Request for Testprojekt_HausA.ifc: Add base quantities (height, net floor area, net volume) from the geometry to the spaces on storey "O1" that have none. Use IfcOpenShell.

First a look at what the model holds.

```python
import ifcopenshell
import ifcopenshell.util.element
import ifcopenshell.util.unit

model = ifcopenshell.open("Testprojekt_HausA.ifc")
print(model.schema)
for unit_type in ("LENGTHUNIT", "AREAUNIT", "VOLUMEUNIT"):
    print(unit_type, ifcopenshell.util.unit.calculate_unit_scale(model, unit_type))
storey = next(s for s in model.by_type("IfcBuildingStorey") if s.Name == "O1")
spaces = [e for e in ifcopenshell.util.element.get_decomposition(storey) if e.is_a("IfcSpace")]
for e in sorted(spaces, key=lambda e: e.id()):
    print(e.id(), e.is_a(), e.Name, list(ifcopenshell.util.element.get_psets(e, qtos_only=True)), sep=" | ")
```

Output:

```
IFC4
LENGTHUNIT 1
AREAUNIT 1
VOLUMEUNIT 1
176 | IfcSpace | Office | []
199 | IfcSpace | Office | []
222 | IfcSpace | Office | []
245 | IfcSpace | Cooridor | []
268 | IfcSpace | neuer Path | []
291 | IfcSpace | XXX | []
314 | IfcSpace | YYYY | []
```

```python
import ifcopenshell
import ifcopenshell.api.pset
import ifcopenshell.geom
import ifcopenshell.util.element
import ifcopenshell.util.shape
import ifcopenshell.util.unit

model = ifcopenshell.open("Testprojekt_HausA.ifc")
unit_scale = ifcopenshell.util.unit.calculate_unit_scale(model)
area_scale = ifcopenshell.util.unit.calculate_unit_scale(model, "AREAUNIT")
volume_scale = ifcopenshell.util.unit.calculate_unit_scale(model, "VOLUMEUNIT")
settings = ifcopenshell.geom.settings()

storey = next(s for s in model.by_type("IfcBuildingStorey") if s.Name == "O1")
spaces = [e for e in ifcopenshell.util.element.get_decomposition(storey) if e.is_a("IfcSpace")]

for e in sorted(spaces, key=lambda e: e.id()):
    if ifcopenshell.util.element.get_psets(e, qtos_only=True, should_inherit=False):
        continue
    # Geometry comes back in metres, in the element's own axes.
    shape = ifcopenshell.geom.create_shape(settings, e)
    values = {
        "Height": ifcopenshell.util.shape.get_z(shape.geometry) / unit_scale,
        "NetFloorArea": ifcopenshell.util.shape.get_footprint_area(shape.geometry) / area_scale,
        "NetVolume": ifcopenshell.util.shape.get_volume(shape.geometry) / volume_scale,
    }
    qto = ifcopenshell.api.pset.add_qto(model, product=e, name="Qto_SpaceBaseQuantities")
    ifcopenshell.api.pset.edit_qto(model, qto=qto, properties=values)
    print(e.id(), {k: round(v, 3) for k, v in values.items()})

model.write("Testprojekt_HausA_rev.ifc")
```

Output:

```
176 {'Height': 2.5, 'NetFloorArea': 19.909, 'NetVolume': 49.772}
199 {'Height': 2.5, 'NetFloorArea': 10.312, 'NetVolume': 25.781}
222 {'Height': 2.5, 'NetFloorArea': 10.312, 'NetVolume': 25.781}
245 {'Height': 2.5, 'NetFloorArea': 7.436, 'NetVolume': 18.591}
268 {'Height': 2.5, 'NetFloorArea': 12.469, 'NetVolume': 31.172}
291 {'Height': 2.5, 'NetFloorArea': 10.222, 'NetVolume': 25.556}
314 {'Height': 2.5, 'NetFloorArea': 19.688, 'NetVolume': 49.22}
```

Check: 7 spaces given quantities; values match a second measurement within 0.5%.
